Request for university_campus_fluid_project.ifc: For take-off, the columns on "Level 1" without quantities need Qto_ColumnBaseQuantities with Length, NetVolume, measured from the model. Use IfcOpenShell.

First a look at what the model holds.

```python
import ifcopenshell
import ifcopenshell.util.element
import ifcopenshell.util.unit

model = ifcopenshell.open("university_campus_fluid_project.ifc")
print(model.schema)
for unit_type in ("LENGTHUNIT", "AREAUNIT", "VOLUMEUNIT"):
    print(unit_type, ifcopenshell.util.unit.calculate_unit_scale(model, unit_type))
storey = next(s for s in model.by_type("IfcBuildingStorey") if s.Name == "Level 1")
columns = [e for e in ifcopenshell.util.element.get_decomposition(storey) if e.is_a("IfcColumn")]
for e in sorted(columns, key=lambda e: e.id()):
    print(e.id(), e.is_a(), e.Name, list(ifcopenshell.util.element.get_psets(e, qtos_only=True)), sep=" | ")
```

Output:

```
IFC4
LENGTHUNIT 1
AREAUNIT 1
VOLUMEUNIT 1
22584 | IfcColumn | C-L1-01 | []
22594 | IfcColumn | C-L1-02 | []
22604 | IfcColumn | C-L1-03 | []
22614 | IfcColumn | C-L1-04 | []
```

```python
import ifcopenshell
import ifcopenshell.api.pset
import ifcopenshell.geom
import ifcopenshell.util.element
import ifcopenshell.util.shape
import ifcopenshell.util.unit

model = ifcopenshell.open("university_campus_fluid_project.ifc")
unit_scale = ifcopenshell.util.unit.calculate_unit_scale(model)
volume_scale = ifcopenshell.util.unit.calculate_unit_scale(model, "VOLUMEUNIT")
settings = ifcopenshell.geom.settings()

storey = next(s for s in model.by_type("IfcBuildingStorey") if s.Name == "Level 1")
columns = [e for e in ifcopenshell.util.element.get_decomposition(storey) if e.is_a("IfcColumn")]

for e in sorted(columns, key=lambda e: e.id()):
    if ifcopenshell.util.element.get_psets(e, qtos_only=True, should_inherit=False):
        continue
    # Geometry comes back in metres, in the element's own axes.
    shape = ifcopenshell.geom.create_shape(settings, e)
    values = {
        "Length": ifcopenshell.util.shape.get_z(shape.geometry) / unit_scale,
        "NetVolume": ifcopenshell.util.shape.get_volume(shape.geometry) / volume_scale,
    }
    qto = ifcopenshell.api.pset.add_qto(model, product=e, name="Qto_ColumnBaseQuantities")
    ifcopenshell.api.pset.edit_qto(model, qto=qto, properties=values)
    print(e.id(), {k: round(v, 3) for k, v in values.items()})

model.write("university_campus_fluid_project-out.ifc")
```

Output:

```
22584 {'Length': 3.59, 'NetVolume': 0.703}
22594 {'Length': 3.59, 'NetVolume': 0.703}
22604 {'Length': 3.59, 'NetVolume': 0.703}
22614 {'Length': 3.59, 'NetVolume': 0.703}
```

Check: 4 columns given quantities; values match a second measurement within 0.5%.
